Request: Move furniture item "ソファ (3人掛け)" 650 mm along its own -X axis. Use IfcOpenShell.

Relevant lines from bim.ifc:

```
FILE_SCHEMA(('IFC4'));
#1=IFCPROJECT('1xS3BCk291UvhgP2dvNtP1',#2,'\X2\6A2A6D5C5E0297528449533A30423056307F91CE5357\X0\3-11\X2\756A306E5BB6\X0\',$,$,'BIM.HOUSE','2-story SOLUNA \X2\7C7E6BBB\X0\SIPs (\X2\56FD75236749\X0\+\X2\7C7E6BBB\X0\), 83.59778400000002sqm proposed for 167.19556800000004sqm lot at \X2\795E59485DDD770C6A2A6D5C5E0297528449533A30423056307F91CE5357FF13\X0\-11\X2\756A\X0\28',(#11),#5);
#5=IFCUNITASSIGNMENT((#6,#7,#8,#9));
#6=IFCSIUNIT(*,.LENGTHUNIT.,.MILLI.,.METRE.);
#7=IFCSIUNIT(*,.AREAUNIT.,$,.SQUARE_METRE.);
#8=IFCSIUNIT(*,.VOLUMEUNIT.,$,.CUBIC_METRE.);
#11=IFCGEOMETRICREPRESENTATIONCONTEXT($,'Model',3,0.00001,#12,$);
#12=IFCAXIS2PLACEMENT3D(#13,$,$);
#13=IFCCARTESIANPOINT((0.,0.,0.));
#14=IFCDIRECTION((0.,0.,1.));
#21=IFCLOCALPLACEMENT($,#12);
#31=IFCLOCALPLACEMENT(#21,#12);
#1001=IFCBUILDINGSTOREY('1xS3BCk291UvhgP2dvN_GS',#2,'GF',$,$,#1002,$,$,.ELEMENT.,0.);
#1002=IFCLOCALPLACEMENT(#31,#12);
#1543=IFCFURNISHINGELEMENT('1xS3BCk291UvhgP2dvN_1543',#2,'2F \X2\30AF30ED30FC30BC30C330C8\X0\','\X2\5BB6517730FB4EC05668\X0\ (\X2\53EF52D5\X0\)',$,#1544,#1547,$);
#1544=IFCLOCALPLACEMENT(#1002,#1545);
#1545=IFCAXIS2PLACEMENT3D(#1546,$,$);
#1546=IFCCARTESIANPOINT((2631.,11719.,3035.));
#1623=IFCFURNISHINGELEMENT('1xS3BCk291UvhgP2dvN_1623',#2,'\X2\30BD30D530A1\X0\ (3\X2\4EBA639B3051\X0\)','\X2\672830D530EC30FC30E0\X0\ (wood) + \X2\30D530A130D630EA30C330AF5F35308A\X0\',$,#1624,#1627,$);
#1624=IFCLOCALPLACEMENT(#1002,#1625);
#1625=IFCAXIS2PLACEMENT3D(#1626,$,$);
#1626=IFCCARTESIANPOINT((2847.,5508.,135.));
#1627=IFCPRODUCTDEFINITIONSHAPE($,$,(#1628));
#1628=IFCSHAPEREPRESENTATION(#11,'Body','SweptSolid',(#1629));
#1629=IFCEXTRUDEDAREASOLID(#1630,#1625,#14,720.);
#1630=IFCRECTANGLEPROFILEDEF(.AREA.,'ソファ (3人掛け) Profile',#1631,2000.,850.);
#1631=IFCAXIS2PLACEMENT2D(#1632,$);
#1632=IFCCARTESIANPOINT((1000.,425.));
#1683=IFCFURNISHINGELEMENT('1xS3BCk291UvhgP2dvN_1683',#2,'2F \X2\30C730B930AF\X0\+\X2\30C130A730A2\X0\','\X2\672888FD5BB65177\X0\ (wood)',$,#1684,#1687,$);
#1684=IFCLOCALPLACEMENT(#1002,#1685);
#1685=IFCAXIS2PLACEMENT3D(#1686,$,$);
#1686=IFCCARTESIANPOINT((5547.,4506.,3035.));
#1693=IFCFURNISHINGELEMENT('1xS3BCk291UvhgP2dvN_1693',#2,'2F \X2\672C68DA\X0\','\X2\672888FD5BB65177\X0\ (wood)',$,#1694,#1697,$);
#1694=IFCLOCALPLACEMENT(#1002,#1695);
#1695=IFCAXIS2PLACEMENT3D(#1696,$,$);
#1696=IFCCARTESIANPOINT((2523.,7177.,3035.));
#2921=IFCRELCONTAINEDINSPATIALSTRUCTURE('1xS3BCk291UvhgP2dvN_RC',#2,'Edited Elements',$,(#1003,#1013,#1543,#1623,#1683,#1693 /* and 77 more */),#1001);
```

```python
import ifcopenshell
import ifcopenshell.api.geometry
import ifcopenshell.util.placement
import ifcopenshell.util.unit

model = ifcopenshell.open("bim.ifc")
unit_scale = ifcopenshell.util.unit.calculate_unit_scale(model)

item = model.by_id(1623)
matrix = ifcopenshell.util.placement.get_local_placement(item.ObjectPlacement)
matrix[:3, 3] -= matrix[:3, 0] * 0.65 / unit_scale
ifcopenshell.api.geometry.edit_object_placement(model, product=item, matrix=matrix, is_si=False)

print(ifcopenshell.util.placement.get_local_placement(item.ObjectPlacement).round(3) + 0.0)

model.write("bim_rev.ifc")
```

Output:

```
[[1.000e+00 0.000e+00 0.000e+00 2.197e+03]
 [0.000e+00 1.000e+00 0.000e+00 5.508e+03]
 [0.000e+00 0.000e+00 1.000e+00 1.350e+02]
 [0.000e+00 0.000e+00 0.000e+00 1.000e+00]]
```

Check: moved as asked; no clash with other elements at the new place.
